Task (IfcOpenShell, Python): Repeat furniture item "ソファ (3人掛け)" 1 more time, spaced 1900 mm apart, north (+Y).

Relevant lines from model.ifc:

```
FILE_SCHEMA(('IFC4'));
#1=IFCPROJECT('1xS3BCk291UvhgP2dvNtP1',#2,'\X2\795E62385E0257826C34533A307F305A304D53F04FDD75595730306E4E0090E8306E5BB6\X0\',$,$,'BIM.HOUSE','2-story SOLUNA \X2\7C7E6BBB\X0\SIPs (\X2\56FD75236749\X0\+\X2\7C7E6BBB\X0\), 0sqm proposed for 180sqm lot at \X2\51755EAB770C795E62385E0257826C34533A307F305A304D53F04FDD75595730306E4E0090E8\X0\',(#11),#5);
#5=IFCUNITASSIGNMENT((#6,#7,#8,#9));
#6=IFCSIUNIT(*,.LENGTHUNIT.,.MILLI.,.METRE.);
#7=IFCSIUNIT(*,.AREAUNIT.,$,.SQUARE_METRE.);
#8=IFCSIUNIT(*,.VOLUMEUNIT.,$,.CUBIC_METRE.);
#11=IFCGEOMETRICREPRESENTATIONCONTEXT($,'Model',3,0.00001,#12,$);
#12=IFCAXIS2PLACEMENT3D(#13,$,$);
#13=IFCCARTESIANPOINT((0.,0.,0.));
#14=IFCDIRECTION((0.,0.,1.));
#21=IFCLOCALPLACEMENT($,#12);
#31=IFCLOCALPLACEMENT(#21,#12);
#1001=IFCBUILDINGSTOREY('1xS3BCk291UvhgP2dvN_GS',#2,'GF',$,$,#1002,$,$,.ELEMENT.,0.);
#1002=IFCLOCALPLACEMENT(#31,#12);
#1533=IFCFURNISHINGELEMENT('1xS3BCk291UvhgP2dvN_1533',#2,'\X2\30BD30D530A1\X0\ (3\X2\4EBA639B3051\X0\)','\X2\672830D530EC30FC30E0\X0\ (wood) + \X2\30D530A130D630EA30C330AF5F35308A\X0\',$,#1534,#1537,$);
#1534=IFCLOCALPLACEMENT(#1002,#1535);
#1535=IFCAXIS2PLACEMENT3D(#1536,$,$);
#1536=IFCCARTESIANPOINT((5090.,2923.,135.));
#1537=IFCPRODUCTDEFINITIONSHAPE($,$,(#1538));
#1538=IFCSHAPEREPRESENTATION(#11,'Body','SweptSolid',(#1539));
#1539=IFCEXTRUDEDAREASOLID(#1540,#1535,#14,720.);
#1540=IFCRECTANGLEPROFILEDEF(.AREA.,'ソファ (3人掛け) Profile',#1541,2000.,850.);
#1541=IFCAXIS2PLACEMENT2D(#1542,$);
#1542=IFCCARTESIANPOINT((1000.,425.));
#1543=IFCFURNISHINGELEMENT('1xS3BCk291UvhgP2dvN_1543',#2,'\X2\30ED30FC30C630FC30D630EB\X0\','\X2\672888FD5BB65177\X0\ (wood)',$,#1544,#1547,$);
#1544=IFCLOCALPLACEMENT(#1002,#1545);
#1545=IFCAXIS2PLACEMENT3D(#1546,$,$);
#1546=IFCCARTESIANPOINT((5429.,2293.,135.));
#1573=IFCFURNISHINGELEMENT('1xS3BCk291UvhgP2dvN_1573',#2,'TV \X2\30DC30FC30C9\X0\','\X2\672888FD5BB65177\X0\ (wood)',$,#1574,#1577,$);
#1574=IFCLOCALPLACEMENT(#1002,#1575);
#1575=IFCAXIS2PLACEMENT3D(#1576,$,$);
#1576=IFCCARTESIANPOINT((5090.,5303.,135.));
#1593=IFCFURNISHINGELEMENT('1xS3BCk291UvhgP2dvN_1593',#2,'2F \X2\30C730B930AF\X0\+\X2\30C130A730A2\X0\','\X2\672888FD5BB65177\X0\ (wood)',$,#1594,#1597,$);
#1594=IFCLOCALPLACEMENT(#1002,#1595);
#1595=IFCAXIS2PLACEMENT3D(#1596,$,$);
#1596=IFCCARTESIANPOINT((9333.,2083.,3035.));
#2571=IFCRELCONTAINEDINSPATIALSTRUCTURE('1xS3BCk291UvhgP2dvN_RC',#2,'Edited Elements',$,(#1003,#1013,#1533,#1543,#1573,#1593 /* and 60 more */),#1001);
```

```python
import numpy as np
import ifcopenshell
import ifcopenshell.api.geometry
import ifcopenshell.api.root
import ifcopenshell.util.element
import ifcopenshell.util.placement

model = ifcopenshell.open("model.ifc")


def reuse_history(source, copy):
    """copy_class also copies each property set's owner history, people and application; keep the originals."""
    for rel in copy.IsDefinedBy:
        if rel.is_a("IfcRelDefinesByProperties") and (history := rel.RelatingPropertyDefinition.OwnerHistory):
            rel.RelatingPropertyDefinition.OwnerHistory = source.OwnerHistory
            ifcopenshell.util.element.remove_deep2(model, history)


source = model.by_guid("1xS3BCk291UvhgP2dvN_1533")
base = ifcopenshell.util.placement.get_local_placement(source.ObjectPlacement)
step = np.array([0.0, 1.0, 0.0]) * 1900.0

for i in range(1, 2):
    copy = ifcopenshell.api.root.copy_class(model, product=source)
    copy.Representation = ifcopenshell.util.element.copy_deep(
        model, source.Representation, exclude=["IfcGeometricRepresentationContext", "IfcRepresentationMap"]
    )
    reuse_history(source, copy)
    matrix = base.copy()
    matrix[:3, 3] += i * step
    print("added at", matrix[:3, 3].round(3) + 0.0)
    ifcopenshell.api.geometry.edit_object_placement(model, product=copy, matrix=matrix, is_si=False)

model.write("model-out.ifc")
```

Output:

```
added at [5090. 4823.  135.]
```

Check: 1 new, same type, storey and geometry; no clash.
